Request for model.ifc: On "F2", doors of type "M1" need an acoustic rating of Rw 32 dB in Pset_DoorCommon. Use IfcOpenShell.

First a look at what the model holds.

```python
import ifcopenshell
import ifcopenshell.util.element

model = ifcopenshell.open("model.ifc")
print(model.schema)
storey = next(s for s in model.by_type("IfcBuildingStorey") if s.Name == "F2")
doors = [e for e in ifcopenshell.util.element.get_decomposition(storey) if e.is_a("IfcDoor")]
seen = {}
for e in doors:
    element_type = ifcopenshell.util.element.get_type(e)
    key = (element_type.Name if element_type != e and element_type else None, ifcopenshell.util.element.get_pset(e, "Pset_DoorCommon", "AcousticRating"))
    seen[key] = seen.get(key, 0) + 1
for (name, value), count in sorted(seen.items(), key=str):
    print(count, "x", name, "|", value)
```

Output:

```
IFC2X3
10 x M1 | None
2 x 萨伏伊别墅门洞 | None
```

```python
import ifcopenshell
import ifcopenshell.api.pset
import ifcopenshell.util.element

model = ifcopenshell.open("model.ifc")

storey = next(s for s in model.by_type("IfcBuildingStorey") if s.Name == "F2")
doors = [e for e in ifcopenshell.util.element.get_decomposition(storey) if e.is_a("IfcDoor")]

count = 0
for e in doors:
    element_type = ifcopenshell.util.element.get_type(e)
    if element_type in (None, e) or element_type.Name != "M1":
        continue
    # add_pset returns the element's existing set when there is one.
    pset = ifcopenshell.api.pset.add_pset(model, product=e, name="Pset_DoorCommon")
    ifcopenshell.api.pset.edit_pset(model, pset=pset, properties={"AcousticRating": "Rw 32 dB"})
    count += 1

print(count, "doors updated")

model.write("model_rev.ifc")
```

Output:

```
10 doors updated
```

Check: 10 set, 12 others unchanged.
